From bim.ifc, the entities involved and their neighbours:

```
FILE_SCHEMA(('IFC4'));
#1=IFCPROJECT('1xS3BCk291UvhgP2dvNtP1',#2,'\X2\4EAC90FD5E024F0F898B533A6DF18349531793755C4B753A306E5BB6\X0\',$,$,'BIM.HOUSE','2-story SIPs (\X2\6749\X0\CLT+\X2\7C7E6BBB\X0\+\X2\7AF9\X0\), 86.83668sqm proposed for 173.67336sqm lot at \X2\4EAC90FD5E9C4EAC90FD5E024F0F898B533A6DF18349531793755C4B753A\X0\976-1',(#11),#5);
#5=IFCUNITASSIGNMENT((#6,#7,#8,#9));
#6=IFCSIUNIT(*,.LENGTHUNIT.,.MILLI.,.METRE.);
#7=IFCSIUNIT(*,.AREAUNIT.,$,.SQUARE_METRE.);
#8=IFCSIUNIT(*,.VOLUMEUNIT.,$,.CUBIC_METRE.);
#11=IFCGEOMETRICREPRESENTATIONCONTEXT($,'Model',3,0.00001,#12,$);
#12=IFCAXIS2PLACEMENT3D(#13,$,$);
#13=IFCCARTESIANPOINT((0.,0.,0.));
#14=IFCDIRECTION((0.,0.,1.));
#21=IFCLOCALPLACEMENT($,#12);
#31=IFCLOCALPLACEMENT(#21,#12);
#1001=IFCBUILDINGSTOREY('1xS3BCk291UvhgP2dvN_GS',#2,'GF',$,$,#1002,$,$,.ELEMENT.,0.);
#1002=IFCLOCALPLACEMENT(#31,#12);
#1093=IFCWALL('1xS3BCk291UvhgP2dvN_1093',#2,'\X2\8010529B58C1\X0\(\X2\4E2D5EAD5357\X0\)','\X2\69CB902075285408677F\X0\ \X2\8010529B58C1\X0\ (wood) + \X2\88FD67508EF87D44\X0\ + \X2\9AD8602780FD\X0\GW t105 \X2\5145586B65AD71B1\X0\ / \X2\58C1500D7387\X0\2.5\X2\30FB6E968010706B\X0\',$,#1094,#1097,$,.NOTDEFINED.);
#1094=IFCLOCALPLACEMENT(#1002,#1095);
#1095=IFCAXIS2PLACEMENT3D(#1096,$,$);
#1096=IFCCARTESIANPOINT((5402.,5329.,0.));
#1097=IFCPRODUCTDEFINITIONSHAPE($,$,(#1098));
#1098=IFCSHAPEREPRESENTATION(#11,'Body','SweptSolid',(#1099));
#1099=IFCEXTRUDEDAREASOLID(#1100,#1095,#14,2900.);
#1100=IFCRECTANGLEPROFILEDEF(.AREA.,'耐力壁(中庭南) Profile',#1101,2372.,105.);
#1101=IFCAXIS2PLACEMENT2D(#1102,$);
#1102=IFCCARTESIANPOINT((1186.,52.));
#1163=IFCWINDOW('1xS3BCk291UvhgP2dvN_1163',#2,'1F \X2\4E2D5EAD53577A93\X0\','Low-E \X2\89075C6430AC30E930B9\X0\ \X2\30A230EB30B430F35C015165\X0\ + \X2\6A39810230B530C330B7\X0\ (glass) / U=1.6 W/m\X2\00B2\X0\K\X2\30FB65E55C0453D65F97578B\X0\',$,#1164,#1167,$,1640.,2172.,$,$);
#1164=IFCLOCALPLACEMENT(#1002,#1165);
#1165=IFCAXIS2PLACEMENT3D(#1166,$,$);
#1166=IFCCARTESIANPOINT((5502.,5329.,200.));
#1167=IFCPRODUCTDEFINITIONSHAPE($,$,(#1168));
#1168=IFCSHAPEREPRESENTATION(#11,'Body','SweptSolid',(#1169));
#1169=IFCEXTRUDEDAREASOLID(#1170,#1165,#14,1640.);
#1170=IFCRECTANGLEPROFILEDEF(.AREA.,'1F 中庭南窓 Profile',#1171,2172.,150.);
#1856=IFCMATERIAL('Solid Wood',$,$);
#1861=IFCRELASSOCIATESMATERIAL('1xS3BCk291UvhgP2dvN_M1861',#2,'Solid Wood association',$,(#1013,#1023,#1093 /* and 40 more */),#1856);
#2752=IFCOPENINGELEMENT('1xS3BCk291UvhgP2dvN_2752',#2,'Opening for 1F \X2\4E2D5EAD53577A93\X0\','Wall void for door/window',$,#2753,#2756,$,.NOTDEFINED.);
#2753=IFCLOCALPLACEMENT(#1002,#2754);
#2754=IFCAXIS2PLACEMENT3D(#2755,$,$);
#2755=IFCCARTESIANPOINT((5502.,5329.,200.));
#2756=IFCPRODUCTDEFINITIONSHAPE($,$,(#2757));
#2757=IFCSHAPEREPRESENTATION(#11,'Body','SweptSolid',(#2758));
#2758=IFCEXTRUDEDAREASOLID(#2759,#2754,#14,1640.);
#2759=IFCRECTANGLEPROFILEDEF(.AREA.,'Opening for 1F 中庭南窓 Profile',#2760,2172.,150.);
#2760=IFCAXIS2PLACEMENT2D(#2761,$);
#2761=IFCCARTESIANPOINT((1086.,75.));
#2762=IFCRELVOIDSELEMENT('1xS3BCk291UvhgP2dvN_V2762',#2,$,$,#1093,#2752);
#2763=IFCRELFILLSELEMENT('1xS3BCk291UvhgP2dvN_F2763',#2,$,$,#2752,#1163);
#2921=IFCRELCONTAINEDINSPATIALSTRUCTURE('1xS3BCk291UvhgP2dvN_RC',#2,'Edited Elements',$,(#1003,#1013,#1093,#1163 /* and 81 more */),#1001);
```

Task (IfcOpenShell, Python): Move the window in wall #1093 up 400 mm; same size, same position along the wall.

```python
import numpy as np
import ifcopenshell
import ifcopenshell.api.geometry
import ifcopenshell.util.placement
import ifcopenshell.util.unit

model = ifcopenshell.open("bim.ifc")
unit_scale = ifcopenshell.util.unit.calculate_unit_scale(model)

window = model.by_guid("1xS3BCk291UvhgP2dvN_1163")
opening = window.FillsVoids[0].RelatingOpeningElement
dz = 400.0

shift = np.array([0.0, 0.0, dz])
# The window is not placed relative to its opening, so move both.
for product in (opening, window):
    matrix = ifcopenshell.util.placement.get_local_placement(product.ObjectPlacement)
    matrix[:3, 3] += shift
    ifcopenshell.api.geometry.edit_object_placement(model, product=product, matrix=matrix, is_si=False)

print(f"moved by {dz * unit_scale:+.3f} m")

model.write("bim_v2.ifc")
```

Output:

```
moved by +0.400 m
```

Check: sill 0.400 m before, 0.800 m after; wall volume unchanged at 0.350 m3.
